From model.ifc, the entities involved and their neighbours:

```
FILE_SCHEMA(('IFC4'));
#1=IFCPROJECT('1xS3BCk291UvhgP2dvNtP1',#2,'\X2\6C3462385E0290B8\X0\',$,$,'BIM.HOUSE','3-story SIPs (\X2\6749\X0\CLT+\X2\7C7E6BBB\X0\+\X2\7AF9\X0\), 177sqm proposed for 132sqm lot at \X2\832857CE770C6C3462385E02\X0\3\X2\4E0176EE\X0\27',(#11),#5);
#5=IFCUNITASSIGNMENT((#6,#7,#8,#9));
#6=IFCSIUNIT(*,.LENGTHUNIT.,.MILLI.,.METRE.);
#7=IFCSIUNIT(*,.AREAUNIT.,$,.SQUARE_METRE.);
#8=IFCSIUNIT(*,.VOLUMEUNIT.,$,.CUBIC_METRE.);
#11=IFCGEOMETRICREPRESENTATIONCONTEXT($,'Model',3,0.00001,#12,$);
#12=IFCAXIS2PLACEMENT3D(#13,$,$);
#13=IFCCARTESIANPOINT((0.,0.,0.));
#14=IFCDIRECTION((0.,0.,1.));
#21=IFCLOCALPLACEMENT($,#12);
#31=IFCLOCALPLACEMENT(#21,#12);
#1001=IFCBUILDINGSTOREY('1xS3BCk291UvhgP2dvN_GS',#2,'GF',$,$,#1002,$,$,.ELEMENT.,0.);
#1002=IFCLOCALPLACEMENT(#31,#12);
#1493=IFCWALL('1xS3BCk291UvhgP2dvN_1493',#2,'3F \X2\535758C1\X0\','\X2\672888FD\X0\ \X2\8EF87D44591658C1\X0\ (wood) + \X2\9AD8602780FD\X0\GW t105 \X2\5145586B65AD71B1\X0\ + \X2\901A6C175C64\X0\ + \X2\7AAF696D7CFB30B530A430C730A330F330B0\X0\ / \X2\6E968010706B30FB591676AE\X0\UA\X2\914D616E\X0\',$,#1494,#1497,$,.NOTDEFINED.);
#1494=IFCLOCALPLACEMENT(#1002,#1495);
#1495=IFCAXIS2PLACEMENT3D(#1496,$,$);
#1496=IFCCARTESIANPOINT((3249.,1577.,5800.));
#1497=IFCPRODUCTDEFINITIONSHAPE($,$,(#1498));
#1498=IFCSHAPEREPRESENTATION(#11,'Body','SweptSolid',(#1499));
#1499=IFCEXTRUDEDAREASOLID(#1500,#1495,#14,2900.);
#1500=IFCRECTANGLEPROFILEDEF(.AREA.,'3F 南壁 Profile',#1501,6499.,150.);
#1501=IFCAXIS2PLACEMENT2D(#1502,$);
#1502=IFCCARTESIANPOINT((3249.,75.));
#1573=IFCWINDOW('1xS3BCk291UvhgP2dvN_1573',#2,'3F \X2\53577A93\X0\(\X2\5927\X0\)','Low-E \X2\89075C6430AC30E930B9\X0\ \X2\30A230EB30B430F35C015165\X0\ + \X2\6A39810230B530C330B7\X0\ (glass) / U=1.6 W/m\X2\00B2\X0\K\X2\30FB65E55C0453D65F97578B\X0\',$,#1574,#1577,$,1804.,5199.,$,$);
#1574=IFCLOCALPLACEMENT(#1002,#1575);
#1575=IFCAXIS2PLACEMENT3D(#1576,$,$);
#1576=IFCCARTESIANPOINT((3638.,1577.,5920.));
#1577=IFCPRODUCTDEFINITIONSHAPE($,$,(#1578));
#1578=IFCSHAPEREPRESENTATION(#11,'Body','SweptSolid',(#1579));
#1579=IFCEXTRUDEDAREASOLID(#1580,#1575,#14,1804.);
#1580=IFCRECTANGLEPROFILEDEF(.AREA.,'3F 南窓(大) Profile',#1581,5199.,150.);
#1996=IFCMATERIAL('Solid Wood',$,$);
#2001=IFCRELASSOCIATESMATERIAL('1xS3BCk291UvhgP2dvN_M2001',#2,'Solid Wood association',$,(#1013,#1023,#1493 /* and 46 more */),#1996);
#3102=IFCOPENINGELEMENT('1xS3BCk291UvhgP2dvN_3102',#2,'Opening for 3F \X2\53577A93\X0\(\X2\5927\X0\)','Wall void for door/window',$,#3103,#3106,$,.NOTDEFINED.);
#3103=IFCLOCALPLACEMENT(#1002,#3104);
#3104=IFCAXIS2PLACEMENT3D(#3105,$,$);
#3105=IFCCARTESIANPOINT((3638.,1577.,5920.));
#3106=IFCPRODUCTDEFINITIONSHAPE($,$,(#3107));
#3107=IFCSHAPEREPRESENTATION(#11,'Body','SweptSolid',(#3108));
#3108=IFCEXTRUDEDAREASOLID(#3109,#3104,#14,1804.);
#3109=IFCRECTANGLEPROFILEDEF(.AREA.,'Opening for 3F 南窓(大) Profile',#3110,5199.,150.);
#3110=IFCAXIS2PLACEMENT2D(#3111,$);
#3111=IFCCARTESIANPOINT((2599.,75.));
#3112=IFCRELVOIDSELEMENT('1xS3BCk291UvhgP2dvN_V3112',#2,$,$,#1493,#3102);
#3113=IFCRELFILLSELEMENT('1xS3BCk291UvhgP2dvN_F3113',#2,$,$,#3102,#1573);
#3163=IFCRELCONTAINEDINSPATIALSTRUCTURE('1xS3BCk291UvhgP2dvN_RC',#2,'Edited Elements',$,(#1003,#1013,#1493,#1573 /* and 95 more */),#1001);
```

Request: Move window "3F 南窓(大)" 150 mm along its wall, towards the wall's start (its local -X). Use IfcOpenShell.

```python
import ifcopenshell
import ifcopenshell.api.geometry
import ifcopenshell.util.placement
import ifcopenshell.util.unit

model = ifcopenshell.open("model.ifc")
unit_scale = ifcopenshell.util.unit.calculate_unit_scale(model)

window = model.by_guid("1xS3BCk291UvhgP2dvN_1573")
opening = window.FillsVoids[0].RelatingOpeningElement
wall = opening.VoidsElements[0].RelatingBuildingElement

wall_matrix = ifcopenshell.util.placement.get_local_placement(wall.ObjectPlacement)
shift = wall_matrix[:3, 0] * -0.15 / unit_scale
before = ifcopenshell.util.placement.get_local_placement(window.ObjectPlacement)[:3, 3].copy()

# The window is not placed relative to its opening, so move both.
for product in (opening, window):
    matrix = ifcopenshell.util.placement.get_local_placement(product.ObjectPlacement)
    matrix[:3, 3] += shift
    ifcopenshell.api.geometry.edit_object_placement(model, product=product, matrix=matrix, is_si=False)

after = ifcopenshell.util.placement.get_local_placement(window.ObjectPlacement)[:3, 3]
print("window moved by", (after - before).round(3) + 0.0)

model.write("model_rev.ifc")
```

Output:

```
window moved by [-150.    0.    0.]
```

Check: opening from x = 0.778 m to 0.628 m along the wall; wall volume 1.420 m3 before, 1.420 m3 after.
